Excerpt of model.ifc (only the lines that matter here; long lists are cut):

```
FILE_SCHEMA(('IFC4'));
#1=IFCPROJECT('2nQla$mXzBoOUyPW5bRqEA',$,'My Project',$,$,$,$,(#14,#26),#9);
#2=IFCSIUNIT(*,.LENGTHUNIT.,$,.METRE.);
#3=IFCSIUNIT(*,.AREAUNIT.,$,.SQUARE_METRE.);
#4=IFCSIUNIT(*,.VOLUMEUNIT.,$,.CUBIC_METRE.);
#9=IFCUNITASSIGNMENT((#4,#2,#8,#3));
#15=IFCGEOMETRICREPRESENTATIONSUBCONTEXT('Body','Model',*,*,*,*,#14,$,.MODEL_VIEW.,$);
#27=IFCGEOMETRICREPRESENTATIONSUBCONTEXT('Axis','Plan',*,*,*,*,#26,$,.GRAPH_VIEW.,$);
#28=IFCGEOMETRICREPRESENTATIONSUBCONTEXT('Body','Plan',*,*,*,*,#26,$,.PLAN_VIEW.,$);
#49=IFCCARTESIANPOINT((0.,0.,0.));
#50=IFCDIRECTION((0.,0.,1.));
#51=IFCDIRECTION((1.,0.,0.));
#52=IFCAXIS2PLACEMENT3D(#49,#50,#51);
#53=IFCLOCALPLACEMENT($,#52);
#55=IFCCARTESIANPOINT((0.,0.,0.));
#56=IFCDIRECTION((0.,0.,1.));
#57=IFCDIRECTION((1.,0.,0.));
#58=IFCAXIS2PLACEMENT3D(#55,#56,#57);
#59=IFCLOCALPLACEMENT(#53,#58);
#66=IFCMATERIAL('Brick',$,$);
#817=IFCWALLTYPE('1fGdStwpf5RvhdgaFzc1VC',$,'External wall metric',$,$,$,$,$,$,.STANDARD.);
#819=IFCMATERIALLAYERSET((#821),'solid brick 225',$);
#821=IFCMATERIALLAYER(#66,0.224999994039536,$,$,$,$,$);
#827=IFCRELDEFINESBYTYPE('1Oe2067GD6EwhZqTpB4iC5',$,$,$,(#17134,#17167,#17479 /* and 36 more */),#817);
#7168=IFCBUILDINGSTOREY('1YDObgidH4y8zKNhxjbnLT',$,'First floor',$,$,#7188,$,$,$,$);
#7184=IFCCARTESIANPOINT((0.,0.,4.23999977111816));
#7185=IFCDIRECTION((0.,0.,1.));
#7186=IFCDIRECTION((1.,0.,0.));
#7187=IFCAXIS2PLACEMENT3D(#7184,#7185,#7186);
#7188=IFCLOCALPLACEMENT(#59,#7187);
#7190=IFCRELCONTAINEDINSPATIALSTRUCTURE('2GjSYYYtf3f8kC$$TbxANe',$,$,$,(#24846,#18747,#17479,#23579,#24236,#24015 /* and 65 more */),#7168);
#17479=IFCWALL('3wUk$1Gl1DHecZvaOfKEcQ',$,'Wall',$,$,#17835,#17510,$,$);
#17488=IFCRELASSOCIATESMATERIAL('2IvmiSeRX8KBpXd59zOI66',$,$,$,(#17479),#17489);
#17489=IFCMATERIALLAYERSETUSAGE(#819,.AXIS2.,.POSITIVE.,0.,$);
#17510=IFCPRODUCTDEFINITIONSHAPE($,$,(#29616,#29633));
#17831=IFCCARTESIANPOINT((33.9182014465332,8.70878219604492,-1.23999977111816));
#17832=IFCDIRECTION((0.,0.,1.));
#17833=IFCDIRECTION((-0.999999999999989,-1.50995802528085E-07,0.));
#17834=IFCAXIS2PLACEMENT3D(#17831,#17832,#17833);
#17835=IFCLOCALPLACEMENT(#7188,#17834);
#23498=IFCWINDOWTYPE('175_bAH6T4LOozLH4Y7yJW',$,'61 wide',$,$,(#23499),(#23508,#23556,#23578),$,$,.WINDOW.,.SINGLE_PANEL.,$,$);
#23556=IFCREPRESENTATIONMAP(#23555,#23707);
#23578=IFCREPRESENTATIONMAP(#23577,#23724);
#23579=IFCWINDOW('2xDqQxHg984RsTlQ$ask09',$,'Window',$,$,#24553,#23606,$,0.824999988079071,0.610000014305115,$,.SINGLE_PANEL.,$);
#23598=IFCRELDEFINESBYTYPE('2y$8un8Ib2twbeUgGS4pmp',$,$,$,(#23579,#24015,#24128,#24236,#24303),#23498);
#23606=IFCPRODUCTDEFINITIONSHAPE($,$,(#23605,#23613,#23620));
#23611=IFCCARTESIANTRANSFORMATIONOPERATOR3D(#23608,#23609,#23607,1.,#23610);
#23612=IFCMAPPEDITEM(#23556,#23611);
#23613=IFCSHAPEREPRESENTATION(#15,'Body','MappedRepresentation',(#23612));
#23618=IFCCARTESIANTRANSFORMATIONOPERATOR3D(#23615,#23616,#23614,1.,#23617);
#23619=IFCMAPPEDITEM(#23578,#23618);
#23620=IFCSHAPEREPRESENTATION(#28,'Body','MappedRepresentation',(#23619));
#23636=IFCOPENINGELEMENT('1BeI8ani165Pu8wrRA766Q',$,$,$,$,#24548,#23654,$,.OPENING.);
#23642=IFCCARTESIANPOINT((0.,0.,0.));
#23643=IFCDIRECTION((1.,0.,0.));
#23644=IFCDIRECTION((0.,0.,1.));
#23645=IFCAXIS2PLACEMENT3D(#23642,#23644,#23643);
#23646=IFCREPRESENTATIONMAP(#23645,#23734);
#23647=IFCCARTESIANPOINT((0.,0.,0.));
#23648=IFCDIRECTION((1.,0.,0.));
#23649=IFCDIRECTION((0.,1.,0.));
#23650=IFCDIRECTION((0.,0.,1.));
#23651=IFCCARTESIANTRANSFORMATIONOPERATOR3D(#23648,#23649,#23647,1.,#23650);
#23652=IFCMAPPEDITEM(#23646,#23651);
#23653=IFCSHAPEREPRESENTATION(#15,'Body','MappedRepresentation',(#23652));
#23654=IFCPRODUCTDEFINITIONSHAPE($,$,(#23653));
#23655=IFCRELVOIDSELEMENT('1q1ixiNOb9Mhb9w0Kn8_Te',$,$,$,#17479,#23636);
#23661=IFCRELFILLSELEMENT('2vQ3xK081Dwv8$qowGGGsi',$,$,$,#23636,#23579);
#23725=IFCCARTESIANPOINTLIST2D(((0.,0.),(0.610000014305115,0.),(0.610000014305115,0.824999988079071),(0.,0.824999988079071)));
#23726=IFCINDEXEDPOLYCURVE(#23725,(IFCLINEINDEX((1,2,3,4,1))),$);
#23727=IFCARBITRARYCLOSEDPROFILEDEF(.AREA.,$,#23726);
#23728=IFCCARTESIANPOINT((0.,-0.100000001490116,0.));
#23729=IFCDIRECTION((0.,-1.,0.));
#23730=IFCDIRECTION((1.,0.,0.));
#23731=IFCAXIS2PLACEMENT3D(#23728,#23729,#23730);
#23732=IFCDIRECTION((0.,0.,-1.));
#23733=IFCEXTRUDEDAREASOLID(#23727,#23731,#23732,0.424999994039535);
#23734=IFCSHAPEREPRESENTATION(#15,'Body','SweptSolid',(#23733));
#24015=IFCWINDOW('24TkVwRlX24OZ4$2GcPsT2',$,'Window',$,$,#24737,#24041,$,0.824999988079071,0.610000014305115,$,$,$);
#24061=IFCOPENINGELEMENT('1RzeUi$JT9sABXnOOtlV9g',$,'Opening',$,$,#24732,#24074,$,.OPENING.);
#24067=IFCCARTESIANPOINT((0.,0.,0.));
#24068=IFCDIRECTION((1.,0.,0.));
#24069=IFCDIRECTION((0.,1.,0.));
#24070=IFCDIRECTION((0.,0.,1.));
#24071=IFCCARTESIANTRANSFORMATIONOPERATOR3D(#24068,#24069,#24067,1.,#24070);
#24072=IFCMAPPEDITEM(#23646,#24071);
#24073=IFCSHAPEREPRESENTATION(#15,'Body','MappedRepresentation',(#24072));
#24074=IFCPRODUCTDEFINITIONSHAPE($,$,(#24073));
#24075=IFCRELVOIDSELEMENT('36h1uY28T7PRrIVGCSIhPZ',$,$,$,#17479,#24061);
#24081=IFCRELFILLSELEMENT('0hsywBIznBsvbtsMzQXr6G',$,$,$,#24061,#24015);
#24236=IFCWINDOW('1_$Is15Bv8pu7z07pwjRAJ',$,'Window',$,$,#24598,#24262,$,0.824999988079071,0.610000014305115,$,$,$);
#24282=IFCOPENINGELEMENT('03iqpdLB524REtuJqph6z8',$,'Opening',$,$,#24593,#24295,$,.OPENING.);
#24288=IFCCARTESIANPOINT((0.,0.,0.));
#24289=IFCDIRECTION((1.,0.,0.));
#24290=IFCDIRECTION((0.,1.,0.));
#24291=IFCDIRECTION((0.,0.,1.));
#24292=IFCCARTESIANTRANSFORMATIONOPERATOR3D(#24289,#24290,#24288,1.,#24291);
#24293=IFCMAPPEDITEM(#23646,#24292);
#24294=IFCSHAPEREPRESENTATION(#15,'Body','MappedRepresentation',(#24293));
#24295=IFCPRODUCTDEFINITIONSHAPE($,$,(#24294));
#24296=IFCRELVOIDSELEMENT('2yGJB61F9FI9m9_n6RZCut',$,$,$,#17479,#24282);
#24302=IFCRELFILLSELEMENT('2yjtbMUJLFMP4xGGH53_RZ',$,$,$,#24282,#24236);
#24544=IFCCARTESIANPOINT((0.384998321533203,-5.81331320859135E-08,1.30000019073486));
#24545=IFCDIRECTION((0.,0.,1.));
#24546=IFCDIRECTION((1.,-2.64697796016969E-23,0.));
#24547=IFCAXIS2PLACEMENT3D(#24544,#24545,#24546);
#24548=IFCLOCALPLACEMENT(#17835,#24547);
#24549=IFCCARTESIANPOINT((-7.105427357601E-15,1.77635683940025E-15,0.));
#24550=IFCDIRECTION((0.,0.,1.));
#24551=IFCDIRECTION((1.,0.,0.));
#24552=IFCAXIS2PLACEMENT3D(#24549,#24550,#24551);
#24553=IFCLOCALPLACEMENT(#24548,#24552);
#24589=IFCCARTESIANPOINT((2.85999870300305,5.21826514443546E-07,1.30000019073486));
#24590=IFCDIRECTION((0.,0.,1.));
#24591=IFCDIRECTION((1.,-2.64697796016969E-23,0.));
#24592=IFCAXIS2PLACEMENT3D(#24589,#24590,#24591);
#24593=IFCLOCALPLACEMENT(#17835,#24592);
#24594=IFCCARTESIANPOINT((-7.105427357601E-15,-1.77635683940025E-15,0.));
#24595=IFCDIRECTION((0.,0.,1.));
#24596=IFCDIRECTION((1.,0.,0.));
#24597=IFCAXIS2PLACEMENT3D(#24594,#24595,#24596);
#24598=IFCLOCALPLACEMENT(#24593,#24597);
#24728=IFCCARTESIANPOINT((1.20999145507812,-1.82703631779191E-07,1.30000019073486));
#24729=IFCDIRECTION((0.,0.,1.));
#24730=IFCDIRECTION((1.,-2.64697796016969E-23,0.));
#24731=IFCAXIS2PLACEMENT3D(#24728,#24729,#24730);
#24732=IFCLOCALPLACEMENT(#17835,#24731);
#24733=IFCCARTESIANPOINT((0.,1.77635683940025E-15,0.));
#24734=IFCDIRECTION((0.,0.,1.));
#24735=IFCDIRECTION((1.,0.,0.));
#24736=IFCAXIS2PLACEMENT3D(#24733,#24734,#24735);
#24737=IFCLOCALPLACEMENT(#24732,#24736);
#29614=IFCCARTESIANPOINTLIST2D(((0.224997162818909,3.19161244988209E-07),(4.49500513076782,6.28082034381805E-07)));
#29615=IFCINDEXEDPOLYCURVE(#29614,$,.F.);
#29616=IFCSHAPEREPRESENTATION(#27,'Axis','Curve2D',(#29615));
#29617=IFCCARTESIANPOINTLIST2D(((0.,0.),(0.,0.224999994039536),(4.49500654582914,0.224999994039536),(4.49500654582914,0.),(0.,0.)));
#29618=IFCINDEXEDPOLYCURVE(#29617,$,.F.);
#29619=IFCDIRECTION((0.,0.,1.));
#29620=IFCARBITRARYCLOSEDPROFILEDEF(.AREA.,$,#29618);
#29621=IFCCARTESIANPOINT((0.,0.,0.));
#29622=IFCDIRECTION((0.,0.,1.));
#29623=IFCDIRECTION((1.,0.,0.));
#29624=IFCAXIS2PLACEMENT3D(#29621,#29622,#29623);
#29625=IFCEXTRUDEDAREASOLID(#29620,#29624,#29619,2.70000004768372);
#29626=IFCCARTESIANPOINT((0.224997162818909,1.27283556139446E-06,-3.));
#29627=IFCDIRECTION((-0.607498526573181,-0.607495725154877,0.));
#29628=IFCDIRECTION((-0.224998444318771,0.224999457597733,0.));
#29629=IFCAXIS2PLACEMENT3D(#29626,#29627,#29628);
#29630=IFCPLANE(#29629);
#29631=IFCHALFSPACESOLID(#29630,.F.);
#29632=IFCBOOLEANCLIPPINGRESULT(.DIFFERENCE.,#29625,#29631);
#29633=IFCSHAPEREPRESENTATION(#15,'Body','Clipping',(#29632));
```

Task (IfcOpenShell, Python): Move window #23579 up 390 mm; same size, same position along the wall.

```python
import numpy as np
import ifcopenshell
import ifcopenshell.api.geometry
import ifcopenshell.util.placement
import ifcopenshell.util.unit

model = ifcopenshell.open("model.ifc")
unit_scale = ifcopenshell.util.unit.calculate_unit_scale(model)

window = model.by_guid("2xDqQxHg984RsTlQ$ask09")
opening = window.FillsVoids[0].RelatingOpeningElement
dz = 0.39

shift = np.array([0.0, 0.0, dz])
# The window is placed relative to its opening, so it follows when the opening moves.
matrix = ifcopenshell.util.placement.get_local_placement(opening.ObjectPlacement)
matrix[:3, 3] += shift
ifcopenshell.api.geometry.edit_object_placement(
    model, product=opening, matrix=matrix, is_si=False, should_transform_children=True
)

print(f"moved by {dz * unit_scale:+.3f} m")

model.write("model_v2.ifc")
```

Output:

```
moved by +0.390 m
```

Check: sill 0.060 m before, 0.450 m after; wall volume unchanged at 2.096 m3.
